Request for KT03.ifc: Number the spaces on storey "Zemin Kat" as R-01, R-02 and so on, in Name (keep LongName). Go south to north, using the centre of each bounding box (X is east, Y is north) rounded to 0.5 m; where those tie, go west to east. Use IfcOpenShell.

First a look at what the model holds.

```python
import ifcopenshell
import ifcopenshell.util.element
import ifcopenshell.util.placement

model = ifcopenshell.open("KT03.ifc")
print(model.schema)
storey = next(s for s in model.by_type("IfcBuildingStorey") if s.Name == "Zemin Kat")
spaces = [e for e in ifcopenshell.util.element.get_decomposition(storey) if e.is_a("IfcSpace")]
for e in sorted(spaces, key=lambda e: e.id()):
    origin = ifcopenshell.util.placement.get_local_placement(e.ObjectPlacement)[:3, 3]
    print(e.id(), e.Name, e.LongName, origin.round(2) + 0.0, sep=" | ")
```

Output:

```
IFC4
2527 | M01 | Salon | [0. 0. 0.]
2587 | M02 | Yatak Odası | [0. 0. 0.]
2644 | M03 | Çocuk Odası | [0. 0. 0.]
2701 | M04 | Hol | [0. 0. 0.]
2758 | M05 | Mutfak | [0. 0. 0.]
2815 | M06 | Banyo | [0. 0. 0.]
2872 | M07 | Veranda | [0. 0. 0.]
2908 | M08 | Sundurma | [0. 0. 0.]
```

```python
import ifcopenshell
import ifcopenshell.geom
import ifcopenshell.util.element
import ifcopenshell.util.shape

model = ifcopenshell.open("KT03.ifc")
settings = ifcopenshell.geom.settings()
settings.set("use-world-coords", True)


def centre(element):
    shape = ifcopenshell.geom.create_shape(settings, element)
    return ifcopenshell.util.shape.get_bbox_centroid(shape.geometry)


storey = next(s for s in model.by_type("IfcBuildingStorey") if s.Name == "Zemin Kat")
spaces = [e for e in ifcopenshell.util.element.get_decomposition(storey) if e.is_a("IfcSpace")]

# Insertion points can sit at a corner or the storey origin, so sort by the geometry (in metres).
centres = {e: centre(e) for e in spaces}
spaces.sort(key=lambda e: (round(centres[e][1] / 0.5), centres[e][0]))

for i, e in enumerate(spaces, start=1):
    number = f"R-{i:02d}"
    e.Name = number
    print(e.id(), number)

model.write("KT03_v2.ifc")
```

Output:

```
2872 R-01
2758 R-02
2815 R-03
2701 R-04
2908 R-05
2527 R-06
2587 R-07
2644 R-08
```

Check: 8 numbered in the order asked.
